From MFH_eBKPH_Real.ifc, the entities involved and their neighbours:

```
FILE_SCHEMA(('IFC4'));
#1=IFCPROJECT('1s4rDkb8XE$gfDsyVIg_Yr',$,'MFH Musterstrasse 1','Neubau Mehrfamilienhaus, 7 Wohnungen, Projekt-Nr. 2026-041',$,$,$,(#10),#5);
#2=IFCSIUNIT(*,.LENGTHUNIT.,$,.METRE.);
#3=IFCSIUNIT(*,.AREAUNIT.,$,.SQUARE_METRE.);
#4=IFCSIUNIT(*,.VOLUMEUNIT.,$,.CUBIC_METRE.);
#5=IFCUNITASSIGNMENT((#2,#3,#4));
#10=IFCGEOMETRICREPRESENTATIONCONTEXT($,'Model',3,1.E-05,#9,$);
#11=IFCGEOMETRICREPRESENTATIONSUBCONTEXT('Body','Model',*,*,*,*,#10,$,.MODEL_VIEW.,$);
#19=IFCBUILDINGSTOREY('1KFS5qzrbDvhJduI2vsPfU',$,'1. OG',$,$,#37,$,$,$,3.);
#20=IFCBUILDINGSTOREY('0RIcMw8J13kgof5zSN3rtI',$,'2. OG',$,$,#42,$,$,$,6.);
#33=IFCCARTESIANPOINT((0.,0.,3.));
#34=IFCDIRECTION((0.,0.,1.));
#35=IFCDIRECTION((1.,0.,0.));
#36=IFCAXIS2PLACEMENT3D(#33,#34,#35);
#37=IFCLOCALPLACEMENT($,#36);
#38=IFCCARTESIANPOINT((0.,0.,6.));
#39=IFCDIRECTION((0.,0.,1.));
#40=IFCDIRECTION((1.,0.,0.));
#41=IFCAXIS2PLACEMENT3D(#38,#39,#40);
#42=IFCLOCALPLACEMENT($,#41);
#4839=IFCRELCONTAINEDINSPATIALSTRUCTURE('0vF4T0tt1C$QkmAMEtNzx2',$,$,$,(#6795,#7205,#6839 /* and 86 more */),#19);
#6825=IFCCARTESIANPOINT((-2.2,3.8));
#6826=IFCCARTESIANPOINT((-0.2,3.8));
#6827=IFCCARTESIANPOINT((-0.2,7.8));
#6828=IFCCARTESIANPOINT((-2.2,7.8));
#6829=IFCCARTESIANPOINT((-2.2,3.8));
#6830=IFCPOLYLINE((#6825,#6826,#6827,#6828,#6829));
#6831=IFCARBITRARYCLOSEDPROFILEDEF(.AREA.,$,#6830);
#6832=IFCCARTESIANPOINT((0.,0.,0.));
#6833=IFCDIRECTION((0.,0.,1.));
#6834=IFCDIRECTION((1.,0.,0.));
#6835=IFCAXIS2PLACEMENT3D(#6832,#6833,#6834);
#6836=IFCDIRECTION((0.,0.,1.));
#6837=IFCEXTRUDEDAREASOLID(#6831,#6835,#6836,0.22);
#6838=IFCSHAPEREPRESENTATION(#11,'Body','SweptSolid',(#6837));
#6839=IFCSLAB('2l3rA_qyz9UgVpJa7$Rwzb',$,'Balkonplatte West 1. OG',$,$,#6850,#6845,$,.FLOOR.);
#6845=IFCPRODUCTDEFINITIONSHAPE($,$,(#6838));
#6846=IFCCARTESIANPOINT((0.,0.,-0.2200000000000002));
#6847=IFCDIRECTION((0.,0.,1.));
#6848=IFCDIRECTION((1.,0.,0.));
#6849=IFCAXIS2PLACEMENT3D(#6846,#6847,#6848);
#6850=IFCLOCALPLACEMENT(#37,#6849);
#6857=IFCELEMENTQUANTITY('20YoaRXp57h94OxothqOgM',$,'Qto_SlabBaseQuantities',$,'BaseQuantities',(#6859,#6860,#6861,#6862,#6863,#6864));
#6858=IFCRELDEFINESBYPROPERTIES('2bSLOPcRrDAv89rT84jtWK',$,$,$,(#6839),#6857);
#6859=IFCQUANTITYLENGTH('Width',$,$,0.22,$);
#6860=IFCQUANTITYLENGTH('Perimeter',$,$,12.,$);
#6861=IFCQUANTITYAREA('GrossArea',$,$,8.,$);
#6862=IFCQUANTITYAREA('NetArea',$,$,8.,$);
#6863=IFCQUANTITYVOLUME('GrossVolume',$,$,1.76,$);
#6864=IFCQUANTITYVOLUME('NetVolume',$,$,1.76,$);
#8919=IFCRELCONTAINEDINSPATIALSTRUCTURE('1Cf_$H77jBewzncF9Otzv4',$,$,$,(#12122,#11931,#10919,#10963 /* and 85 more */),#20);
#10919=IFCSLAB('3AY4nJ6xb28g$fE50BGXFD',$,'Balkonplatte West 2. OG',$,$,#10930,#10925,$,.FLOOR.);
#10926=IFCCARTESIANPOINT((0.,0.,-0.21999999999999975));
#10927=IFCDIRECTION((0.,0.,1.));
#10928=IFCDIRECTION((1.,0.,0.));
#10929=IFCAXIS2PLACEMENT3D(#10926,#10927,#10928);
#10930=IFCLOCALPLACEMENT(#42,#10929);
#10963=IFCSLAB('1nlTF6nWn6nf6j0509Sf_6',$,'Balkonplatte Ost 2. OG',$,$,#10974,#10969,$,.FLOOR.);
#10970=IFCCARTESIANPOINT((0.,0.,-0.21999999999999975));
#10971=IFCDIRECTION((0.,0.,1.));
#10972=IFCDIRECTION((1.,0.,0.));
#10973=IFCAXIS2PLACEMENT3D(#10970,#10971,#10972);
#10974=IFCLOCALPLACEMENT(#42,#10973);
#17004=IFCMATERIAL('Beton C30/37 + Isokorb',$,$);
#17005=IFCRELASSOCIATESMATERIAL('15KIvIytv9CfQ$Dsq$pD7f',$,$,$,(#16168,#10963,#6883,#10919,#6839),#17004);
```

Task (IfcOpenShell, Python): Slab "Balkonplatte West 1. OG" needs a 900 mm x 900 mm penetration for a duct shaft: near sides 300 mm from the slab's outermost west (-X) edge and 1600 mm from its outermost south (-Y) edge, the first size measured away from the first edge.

```python
import numpy as np
import ifcopenshell
import ifcopenshell.api.feature
import ifcopenshell.api.geometry
import ifcopenshell.api.pset
import ifcopenshell.api.root
import ifcopenshell.geom
import ifcopenshell.util.element
import ifcopenshell.util.placement
import ifcopenshell.util.representation
import ifcopenshell.util.shape
import ifcopenshell.util.unit

model = ifcopenshell.open("MFH_eBKPH_Real.ifc")
unit_scale = ifcopenshell.util.unit.calculate_unit_scale(model)
area_scale = ifcopenshell.util.unit.calculate_unit_scale(model, "AREAUNIT")
volume_scale = ifcopenshell.util.unit.calculate_unit_scale(model, "VOLUMEUNIT")
settings = ifcopenshell.geom.settings()


def volume(element):
    """Net volume in cubic metres, openings subtracted."""
    shape = ifcopenshell.geom.create_shape(settings, element)
    return ifcopenshell.util.shape.get_volume(shape.geometry)


slab = model.by_guid("2l3rA_qyz9UgVpJa7$Rwzb")
before = volume(slab)

# Extent in the slab's own axes, in metres. The edges named are its -X and -Y sides.
slab_shape = ifcopenshell.geom.create_shape(settings, slab)
vertices = ifcopenshell.util.shape.get_vertices(slab_shape.geometry)
x_min, y_min, bottom = vertices.min(axis=0)
top = vertices[:, 2].max()

opening = ifcopenshell.api.root.create_entity(model, ifc_class="IfcOpeningElement", name="Duct shaft opening", predefined_type="OPENING")
context = ifcopenshell.util.representation.get_context(model, "Model", "Body", "MODEL_VIEW")
width, depth = 0.9, 0.9
outline = [(0.0, 0.0), (width, 0.0), (width, depth), (0.0, depth), (0.0, 0.0)]
# Overshoot both faces by 50 mm so the cut is clean.
shape = ifcopenshell.api.geometry.add_slab_representation(
    model, context=context, depth=top - bottom + 0.1, polyline=outline
)
ifcopenshell.api.geometry.assign_representation(model, product=opening, representation=shape)

matrix = ifcopenshell.util.placement.get_local_placement(slab.ObjectPlacement)
matrix[:, 3] = matrix @ np.append(np.array([x_min + 0.3, y_min + 1.6, bottom - 0.05]) / unit_scale, 1.0)
ifcopenshell.api.geometry.edit_object_placement(model, product=opening, matrix=matrix, is_si=False)
ifcopenshell.api.feature.add_feature(model, feature=opening, element=slab)

after = volume(slab)

# Update the slab's stored quantities.
qto = model.by_id(ifcopenshell.util.element.get_pset(slab, "Qto_SlabBaseQuantities", should_inherit=False)["id"])
ifcopenshell.api.pset.edit_qto(model, qto=qto, properties={
    "NetArea": after / (top - bottom) / area_scale,
    "NetVolume": after / volume_scale,
})

print(f"slab volume {before:.3f} -> {after:.3f} m3")

model.write("MFH_eBKPH_Real_rev.ifc")
```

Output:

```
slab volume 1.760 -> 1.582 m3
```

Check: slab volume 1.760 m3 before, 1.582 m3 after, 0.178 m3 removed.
